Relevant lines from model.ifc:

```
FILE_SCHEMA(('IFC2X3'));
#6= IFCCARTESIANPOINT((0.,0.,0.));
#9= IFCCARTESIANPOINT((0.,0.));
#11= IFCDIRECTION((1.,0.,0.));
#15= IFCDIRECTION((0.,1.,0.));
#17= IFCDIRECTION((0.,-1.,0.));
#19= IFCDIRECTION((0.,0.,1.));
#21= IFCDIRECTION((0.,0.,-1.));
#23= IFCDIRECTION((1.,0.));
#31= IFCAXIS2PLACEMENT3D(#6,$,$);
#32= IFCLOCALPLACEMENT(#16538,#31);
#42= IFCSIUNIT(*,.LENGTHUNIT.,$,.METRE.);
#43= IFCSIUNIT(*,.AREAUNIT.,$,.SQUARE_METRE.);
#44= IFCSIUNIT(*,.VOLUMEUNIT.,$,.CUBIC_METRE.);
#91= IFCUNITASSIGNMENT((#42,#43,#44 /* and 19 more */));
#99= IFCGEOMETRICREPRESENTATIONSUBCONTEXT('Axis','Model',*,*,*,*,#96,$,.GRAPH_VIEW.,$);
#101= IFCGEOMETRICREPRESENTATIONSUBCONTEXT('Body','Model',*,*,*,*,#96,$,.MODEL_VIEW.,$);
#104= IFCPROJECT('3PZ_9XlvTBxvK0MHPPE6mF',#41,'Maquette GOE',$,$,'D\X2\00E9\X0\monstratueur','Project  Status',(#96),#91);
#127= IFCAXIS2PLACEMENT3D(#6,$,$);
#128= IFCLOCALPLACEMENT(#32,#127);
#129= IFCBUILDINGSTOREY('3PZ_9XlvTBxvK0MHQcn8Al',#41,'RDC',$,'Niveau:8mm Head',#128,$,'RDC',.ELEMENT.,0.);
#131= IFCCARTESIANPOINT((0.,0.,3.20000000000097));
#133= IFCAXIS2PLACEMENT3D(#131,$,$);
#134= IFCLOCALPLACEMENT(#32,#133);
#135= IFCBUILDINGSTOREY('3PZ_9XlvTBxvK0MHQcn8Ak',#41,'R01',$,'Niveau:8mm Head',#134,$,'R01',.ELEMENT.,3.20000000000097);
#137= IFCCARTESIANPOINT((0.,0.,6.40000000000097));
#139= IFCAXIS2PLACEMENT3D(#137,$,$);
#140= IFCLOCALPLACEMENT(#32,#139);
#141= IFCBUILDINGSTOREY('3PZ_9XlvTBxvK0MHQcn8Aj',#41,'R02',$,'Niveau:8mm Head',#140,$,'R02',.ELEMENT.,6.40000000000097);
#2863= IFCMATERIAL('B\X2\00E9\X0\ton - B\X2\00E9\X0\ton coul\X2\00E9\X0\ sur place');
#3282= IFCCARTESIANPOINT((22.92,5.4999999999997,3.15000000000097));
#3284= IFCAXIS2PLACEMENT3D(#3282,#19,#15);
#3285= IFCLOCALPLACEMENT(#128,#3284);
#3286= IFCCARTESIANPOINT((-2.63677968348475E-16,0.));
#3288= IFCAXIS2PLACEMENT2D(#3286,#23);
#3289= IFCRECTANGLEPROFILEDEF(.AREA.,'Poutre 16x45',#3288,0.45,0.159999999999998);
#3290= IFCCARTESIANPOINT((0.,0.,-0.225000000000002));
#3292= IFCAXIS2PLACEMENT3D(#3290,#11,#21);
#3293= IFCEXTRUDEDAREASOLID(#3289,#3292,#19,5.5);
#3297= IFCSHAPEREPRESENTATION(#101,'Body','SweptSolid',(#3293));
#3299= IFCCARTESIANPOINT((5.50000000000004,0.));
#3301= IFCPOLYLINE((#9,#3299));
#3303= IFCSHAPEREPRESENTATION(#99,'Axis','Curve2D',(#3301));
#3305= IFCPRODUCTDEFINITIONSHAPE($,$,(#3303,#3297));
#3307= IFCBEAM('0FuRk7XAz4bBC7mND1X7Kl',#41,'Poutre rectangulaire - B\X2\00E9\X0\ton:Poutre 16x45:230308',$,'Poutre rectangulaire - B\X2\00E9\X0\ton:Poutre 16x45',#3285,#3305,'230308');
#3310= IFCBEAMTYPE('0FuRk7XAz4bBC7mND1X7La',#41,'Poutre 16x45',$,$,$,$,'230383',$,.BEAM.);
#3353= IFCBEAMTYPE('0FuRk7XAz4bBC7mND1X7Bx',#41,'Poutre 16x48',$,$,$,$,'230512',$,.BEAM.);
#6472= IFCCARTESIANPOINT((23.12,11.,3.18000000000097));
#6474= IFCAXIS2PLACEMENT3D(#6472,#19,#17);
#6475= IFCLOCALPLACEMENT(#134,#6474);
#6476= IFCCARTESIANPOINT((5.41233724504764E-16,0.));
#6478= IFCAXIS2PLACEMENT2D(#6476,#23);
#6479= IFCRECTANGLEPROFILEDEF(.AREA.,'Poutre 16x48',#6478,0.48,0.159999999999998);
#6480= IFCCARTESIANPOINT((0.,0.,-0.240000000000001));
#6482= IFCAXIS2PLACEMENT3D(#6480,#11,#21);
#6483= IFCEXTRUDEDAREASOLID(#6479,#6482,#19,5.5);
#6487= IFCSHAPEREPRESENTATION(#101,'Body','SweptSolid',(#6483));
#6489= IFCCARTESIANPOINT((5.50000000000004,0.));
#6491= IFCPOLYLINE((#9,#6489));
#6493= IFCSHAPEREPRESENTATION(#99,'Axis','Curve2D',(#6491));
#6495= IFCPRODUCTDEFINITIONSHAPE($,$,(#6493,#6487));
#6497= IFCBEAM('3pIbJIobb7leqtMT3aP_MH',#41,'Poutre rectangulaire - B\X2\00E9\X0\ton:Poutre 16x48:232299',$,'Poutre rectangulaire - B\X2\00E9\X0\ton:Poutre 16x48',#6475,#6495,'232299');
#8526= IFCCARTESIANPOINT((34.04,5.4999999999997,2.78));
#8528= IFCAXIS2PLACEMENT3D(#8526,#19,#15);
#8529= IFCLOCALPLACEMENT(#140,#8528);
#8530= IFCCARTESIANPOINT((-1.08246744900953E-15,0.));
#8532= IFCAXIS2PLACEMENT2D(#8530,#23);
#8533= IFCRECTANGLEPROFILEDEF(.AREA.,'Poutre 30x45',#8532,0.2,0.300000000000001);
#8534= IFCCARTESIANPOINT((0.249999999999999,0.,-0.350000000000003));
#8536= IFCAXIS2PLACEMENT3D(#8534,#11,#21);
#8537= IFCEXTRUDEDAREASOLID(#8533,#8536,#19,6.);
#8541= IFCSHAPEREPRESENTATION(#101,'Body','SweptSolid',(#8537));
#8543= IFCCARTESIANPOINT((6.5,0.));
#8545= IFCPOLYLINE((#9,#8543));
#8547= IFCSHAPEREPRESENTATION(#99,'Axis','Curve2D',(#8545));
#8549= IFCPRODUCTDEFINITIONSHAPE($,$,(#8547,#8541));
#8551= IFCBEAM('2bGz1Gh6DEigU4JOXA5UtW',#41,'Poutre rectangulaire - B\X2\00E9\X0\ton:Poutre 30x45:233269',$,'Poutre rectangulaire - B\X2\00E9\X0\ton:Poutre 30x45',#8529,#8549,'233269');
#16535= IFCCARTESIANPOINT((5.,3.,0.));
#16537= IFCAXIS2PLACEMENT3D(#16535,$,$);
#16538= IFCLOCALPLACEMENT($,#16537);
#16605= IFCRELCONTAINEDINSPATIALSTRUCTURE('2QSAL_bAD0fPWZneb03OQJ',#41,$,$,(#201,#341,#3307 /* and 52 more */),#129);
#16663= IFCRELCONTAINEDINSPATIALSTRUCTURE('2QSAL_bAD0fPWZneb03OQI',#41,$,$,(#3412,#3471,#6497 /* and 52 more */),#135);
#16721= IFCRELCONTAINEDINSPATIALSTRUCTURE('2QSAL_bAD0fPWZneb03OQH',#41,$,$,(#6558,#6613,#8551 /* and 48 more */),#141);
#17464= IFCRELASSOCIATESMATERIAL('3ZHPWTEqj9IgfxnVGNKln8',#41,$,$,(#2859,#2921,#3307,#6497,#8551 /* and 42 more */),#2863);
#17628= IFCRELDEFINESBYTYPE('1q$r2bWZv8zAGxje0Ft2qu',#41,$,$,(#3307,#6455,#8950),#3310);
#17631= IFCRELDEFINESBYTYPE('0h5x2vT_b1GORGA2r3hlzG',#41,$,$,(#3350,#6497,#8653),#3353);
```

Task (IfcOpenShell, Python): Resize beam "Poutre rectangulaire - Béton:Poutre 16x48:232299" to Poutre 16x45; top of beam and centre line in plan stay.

```python
import ifcopenshell
import ifcopenshell.api.type
import ifcopenshell.util.element
import ifcopenshell.util.representation

model = ifcopenshell.open("model.ifc")

member = model.by_guid("3pIbJIobb7leqtMT3aP_MH")
source = next(p for p in model.by_type("IfcRectangleProfileDef") if p.ProfileName == "Poutre 16x45")

body = ifcopenshell.util.representation.get_representation(member, "Model", "Body")
solid = body.Items[0]
old_profile = solid.SweptArea

# Copy the section's sizes but keep this member's own profile position.
profile = ifcopenshell.util.element.copy(model, source)
# Profiles are centred, so shift by half the change in depth to hold the top.
shift = (old_profile.XDim - profile.XDim) / 2
x, y = old_profile.Position.Location.Coordinates
up = (-1.0, 0.0)  # upwards, in the solid's own plane
location = model.createIfcCartesianPoint((x + up[0] * shift, y + up[1] * shift))
profile.Position = model.createIfcAxis2Placement2D(location, old_profile.Position.RefDirection)
solid.SweptArea = profile
if not model.get_total_inverses(old_profile):
    ifcopenshell.util.element.remove_deep2(model, old_profile)

new_type = model.by_guid("0FuRk7XAz4bBC7mND1X7La")
ifcopenshell.api.type.assign_type(
    model, related_objects=[member], relating_type=new_type, should_map_representations=False
)
member.Name = member.Name.replace("Poutre 16x48", "Poutre 16x45")
member.ObjectType = "Poutre rectangulaire - Béton:Poutre 16x45"

print(solid.SweptArea)

model.write("model_rev.ifc")
```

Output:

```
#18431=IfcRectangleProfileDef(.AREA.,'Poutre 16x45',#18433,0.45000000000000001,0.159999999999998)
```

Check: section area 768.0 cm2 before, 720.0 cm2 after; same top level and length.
